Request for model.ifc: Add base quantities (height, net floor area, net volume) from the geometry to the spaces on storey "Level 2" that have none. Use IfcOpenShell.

First a look at what the model holds.

```python
import ifcopenshell
import ifcopenshell.util.element
import ifcopenshell.util.unit

model = ifcopenshell.open("model.ifc")
print(model.schema)
for unit_type in ("LENGTHUNIT", "AREAUNIT", "VOLUMEUNIT"):
    print(unit_type, ifcopenshell.util.unit.calculate_unit_scale(model, unit_type))
storey = next(s for s in model.by_type("IfcBuildingStorey") if s.Name == "Level 2")
spaces = [e for e in ifcopenshell.util.element.get_decomposition(storey) if e.is_a("IfcSpace")]
for e in sorted(spaces, key=lambda e: e.id()):
    print(e.id(), e.is_a(), e.Name, list(ifcopenshell.util.element.get_psets(e, qtos_only=True)), sep=" | ")
```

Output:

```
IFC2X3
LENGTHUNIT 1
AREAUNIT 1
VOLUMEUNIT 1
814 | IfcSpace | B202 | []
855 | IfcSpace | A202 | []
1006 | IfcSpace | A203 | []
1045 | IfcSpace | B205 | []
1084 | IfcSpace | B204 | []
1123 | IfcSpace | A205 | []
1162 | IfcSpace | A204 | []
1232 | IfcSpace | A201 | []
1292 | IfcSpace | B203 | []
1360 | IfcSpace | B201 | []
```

```python
import ifcopenshell
import ifcopenshell.api.pset
import ifcopenshell.geom
import ifcopenshell.util.element
import ifcopenshell.util.shape
import ifcopenshell.util.unit

model = ifcopenshell.open("model.ifc")
unit_scale = ifcopenshell.util.unit.calculate_unit_scale(model)
area_scale = ifcopenshell.util.unit.calculate_unit_scale(model, "AREAUNIT")
volume_scale = ifcopenshell.util.unit.calculate_unit_scale(model, "VOLUMEUNIT")
settings = ifcopenshell.geom.settings()

storey = next(s for s in model.by_type("IfcBuildingStorey") if s.Name == "Level 2")
spaces = [e for e in ifcopenshell.util.element.get_decomposition(storey) if e.is_a("IfcSpace")]

for e in sorted(spaces, key=lambda e: e.id()):
    if ifcopenshell.util.element.get_psets(e, qtos_only=True, should_inherit=False):
        continue
    # Geometry comes back in metres, in the element's own axes.
    shape = ifcopenshell.geom.create_shape(settings, e)
    values = {
        "Height": ifcopenshell.util.shape.get_z(shape.geometry) / unit_scale,
        "NetFloorArea": ifcopenshell.util.shape.get_footprint_area(shape.geometry) / area_scale,
        "NetVolume": ifcopenshell.util.shape.get_volume(shape.geometry) / volume_scale,
    }
    qto = ifcopenshell.api.pset.add_qto(model, product=e, name="BaseQuantities")
    ifcopenshell.api.pset.edit_qto(model, qto=qto, properties=values)
    print(e.id(), {k: round(v, 3) for k, v in values.items()})

model.write("model_rev.ifc")
```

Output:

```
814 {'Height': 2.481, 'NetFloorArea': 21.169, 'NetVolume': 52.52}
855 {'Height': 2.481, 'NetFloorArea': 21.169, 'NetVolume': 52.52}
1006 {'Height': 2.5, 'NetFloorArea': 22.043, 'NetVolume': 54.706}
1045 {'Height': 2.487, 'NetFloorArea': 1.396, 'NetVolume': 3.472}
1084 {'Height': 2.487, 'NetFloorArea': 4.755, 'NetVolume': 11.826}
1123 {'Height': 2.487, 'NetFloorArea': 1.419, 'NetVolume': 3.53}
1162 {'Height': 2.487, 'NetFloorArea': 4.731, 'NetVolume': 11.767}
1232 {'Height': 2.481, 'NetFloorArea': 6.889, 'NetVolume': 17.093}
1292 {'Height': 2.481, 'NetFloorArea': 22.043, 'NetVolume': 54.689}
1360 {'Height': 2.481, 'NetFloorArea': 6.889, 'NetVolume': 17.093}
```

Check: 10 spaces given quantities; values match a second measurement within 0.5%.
